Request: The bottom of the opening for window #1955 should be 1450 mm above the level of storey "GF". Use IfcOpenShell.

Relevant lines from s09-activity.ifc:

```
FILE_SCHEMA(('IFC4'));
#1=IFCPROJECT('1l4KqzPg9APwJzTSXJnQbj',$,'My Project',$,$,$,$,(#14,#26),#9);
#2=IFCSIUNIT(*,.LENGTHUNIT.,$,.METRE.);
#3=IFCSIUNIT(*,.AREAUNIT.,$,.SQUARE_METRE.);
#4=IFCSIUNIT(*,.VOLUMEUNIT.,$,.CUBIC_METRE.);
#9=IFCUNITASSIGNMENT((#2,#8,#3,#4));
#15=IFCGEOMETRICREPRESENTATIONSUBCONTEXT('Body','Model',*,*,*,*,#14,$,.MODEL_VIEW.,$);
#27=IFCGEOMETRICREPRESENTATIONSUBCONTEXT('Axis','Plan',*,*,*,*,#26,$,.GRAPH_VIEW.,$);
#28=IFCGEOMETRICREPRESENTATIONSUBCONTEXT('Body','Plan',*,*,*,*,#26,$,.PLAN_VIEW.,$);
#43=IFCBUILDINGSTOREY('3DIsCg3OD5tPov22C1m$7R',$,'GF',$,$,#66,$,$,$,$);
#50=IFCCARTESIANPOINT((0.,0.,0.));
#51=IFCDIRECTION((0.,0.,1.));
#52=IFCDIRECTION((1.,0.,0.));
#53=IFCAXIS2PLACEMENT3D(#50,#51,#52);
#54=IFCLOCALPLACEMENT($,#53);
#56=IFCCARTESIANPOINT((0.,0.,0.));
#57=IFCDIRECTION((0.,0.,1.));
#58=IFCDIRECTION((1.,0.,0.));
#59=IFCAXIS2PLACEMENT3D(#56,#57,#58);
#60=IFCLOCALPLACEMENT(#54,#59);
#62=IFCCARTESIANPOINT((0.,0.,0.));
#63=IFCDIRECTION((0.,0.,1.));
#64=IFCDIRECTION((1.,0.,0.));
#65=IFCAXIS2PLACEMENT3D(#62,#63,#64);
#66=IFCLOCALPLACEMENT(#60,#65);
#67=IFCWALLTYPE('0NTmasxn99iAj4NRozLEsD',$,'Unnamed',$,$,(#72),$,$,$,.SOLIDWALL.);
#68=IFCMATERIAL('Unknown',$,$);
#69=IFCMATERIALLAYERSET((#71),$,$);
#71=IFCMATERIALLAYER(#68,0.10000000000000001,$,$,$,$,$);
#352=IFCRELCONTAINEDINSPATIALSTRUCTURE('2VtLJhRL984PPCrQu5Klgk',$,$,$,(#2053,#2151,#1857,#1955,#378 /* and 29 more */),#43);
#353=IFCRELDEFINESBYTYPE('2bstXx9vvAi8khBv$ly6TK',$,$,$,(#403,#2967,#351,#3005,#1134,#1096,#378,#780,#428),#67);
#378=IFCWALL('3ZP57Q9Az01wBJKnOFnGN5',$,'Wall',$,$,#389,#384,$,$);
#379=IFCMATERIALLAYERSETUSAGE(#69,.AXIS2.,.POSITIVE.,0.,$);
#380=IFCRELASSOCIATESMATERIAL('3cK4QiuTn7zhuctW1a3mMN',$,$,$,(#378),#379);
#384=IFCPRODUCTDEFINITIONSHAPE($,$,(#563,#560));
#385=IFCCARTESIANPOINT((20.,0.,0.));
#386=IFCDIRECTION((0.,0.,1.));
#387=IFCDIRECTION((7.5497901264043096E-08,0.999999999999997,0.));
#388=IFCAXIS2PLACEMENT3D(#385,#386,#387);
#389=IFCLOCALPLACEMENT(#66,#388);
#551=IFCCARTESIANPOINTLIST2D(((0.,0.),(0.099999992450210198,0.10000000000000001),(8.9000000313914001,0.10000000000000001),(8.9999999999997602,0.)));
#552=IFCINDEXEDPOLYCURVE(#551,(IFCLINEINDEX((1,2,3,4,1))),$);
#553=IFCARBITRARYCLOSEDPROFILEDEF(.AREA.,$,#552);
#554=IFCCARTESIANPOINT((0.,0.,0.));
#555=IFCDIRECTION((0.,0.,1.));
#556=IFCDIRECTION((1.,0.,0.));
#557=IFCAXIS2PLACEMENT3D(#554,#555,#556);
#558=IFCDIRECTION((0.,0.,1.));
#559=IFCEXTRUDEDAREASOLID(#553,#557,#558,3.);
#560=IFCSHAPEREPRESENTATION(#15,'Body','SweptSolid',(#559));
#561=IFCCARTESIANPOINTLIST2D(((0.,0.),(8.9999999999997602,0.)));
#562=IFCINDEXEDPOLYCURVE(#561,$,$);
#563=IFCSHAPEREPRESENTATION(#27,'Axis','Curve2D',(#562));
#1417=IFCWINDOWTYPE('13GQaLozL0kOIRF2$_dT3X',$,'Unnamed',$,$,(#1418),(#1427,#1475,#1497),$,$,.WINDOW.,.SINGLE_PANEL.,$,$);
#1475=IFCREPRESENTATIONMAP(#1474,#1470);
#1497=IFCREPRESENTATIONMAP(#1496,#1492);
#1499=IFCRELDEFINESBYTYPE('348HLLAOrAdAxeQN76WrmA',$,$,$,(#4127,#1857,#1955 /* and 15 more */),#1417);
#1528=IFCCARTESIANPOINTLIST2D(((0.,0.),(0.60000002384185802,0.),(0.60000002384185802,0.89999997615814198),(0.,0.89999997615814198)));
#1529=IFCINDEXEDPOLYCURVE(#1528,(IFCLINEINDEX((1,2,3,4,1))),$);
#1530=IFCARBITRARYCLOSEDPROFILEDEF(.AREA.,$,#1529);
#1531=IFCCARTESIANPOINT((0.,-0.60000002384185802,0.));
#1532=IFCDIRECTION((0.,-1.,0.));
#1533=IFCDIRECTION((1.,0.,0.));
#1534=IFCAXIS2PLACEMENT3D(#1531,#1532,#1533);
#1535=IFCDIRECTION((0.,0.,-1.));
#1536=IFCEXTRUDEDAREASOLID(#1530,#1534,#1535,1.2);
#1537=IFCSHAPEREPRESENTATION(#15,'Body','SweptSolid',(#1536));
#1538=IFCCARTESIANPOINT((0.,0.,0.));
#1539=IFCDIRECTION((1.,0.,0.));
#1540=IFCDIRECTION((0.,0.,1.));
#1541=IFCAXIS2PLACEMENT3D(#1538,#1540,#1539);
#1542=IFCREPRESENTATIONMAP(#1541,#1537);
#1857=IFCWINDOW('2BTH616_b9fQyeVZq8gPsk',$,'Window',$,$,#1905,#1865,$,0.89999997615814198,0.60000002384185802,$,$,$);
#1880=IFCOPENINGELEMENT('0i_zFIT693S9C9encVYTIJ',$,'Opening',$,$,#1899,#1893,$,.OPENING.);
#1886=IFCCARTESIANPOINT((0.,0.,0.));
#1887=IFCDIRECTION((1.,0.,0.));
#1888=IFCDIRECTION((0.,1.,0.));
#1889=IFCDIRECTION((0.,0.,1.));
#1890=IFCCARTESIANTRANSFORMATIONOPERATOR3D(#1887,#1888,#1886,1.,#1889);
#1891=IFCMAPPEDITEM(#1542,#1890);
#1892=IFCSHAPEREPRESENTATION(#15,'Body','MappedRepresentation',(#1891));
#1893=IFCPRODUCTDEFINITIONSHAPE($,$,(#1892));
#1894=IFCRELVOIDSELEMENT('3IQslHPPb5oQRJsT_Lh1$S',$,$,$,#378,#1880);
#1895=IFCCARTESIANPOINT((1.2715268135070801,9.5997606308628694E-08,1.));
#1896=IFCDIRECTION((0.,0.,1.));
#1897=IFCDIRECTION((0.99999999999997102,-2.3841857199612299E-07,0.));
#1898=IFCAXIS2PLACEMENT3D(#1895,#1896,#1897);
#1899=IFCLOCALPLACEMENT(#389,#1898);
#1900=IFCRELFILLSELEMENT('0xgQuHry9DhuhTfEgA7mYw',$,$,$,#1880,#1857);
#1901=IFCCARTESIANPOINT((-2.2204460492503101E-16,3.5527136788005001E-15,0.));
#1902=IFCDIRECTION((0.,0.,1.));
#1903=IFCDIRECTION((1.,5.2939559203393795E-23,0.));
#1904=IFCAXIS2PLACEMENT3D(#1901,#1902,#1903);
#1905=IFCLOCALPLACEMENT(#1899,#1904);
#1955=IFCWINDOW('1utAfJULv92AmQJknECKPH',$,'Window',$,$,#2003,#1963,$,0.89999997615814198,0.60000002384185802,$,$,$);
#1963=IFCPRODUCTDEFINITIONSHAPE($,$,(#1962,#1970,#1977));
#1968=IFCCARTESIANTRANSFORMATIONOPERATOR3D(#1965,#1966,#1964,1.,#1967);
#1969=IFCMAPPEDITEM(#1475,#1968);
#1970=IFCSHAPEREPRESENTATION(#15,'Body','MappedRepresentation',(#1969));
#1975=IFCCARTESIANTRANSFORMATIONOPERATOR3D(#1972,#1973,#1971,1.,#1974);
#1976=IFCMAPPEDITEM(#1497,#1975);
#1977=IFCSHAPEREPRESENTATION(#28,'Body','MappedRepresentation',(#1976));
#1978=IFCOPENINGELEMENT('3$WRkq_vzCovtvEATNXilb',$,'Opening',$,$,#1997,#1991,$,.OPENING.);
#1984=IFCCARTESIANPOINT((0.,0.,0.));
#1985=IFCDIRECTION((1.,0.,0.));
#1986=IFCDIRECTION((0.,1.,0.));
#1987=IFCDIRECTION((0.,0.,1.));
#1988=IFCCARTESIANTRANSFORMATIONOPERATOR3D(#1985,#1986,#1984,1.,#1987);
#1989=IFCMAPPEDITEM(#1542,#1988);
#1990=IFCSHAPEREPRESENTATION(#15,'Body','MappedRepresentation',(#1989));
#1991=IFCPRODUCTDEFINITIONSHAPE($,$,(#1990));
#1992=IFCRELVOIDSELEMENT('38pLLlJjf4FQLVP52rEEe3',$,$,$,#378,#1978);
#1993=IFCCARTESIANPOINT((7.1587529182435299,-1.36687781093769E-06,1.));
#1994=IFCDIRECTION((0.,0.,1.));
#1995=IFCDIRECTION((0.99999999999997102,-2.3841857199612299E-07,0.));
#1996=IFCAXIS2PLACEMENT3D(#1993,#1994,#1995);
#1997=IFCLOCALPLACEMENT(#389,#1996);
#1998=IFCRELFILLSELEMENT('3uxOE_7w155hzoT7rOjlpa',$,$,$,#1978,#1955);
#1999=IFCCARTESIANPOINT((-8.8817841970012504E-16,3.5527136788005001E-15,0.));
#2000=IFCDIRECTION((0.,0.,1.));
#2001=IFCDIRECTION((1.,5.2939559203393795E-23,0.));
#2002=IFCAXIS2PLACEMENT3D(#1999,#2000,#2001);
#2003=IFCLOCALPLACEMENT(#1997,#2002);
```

```python
import numpy as np
import ifcopenshell
import ifcopenshell.api.geometry
import ifcopenshell.geom
import ifcopenshell.util.element
import ifcopenshell.util.placement
import ifcopenshell.util.shape
import ifcopenshell.util.unit

model = ifcopenshell.open("s09-activity.ifc")
unit_scale = ifcopenshell.util.unit.calculate_unit_scale(model)

window = model.by_guid("1utAfJULv92AmQJknECKPH")
opening = window.FillsVoids[0].RelatingOpeningElement
storey = ifcopenshell.util.element.get_container(window, ifc_class="IfcBuildingStorey")
level = ifcopenshell.util.placement.get_local_placement(storey.ObjectPlacement)[2, 3]

# The opening's origin need not be at the sill, so measure its lowest point.
shape = ifcopenshell.geom.create_shape(ifcopenshell.geom.settings(), opening)
bottom = ifcopenshell.util.shape.get_shape_bottom_elevation(shape, shape.geometry) / unit_scale
dz = level + 1.45 / unit_scale - bottom

shift = np.array([0.0, 0.0, dz])
# The window is placed relative to its opening, so it follows when the opening moves.
matrix = ifcopenshell.util.placement.get_local_placement(opening.ObjectPlacement)
matrix[:3, 3] += shift
ifcopenshell.api.geometry.edit_object_placement(
    model, product=opening, matrix=matrix, is_si=False, should_transform_children=True
)

print(f"moved by {dz * unit_scale:+.3f} m")

model.write("s09-activity_v2.ifc")
```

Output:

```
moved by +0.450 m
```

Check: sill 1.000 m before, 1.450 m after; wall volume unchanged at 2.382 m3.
